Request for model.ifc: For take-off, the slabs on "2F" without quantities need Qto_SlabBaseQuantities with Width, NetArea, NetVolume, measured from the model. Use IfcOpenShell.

First a look at what the model holds.

```python
import ifcopenshell
import ifcopenshell.util.element
import ifcopenshell.util.unit

model = ifcopenshell.open("model.ifc")
print(model.schema)
for unit_type in ("LENGTHUNIT", "AREAUNIT", "VOLUMEUNIT"):
    print(unit_type, ifcopenshell.util.unit.calculate_unit_scale(model, unit_type))
storey = next(s for s in model.by_type("IfcBuildingStorey") if s.Name == "2F")
slabs = [e for e in ifcopenshell.util.element.get_decomposition(storey) if e.is_a("IfcSlab")]
for e in sorted(slabs, key=lambda e: e.id()):
    print(e.id(), e.is_a(), e.Name, list(ifcopenshell.util.element.get_psets(e, qtos_only=True)), sep=" | ")
```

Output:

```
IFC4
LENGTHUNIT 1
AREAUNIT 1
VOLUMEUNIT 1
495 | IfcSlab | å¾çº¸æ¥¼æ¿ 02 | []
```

```python
import ifcopenshell
import ifcopenshell.api.pset
import ifcopenshell.geom
import ifcopenshell.util.element
import ifcopenshell.util.shape
import ifcopenshell.util.unit

model = ifcopenshell.open("model.ifc")
unit_scale = ifcopenshell.util.unit.calculate_unit_scale(model)
area_scale = ifcopenshell.util.unit.calculate_unit_scale(model, "AREAUNIT")
volume_scale = ifcopenshell.util.unit.calculate_unit_scale(model, "VOLUMEUNIT")
settings = ifcopenshell.geom.settings()

storey = next(s for s in model.by_type("IfcBuildingStorey") if s.Name == "2F")
slabs = [e for e in ifcopenshell.util.element.get_decomposition(storey) if e.is_a("IfcSlab")]

for e in sorted(slabs, key=lambda e: e.id()):
    if ifcopenshell.util.element.get_psets(e, qtos_only=True, should_inherit=False):
        continue
    # Geometry comes back in metres, in the element's own axes.
    shape = ifcopenshell.geom.create_shape(settings, e)
    values = {
        "Width": ifcopenshell.util.shape.get_z(shape.geometry) / unit_scale,
        "NetArea": ifcopenshell.util.shape.get_footprint_area(shape.geometry) / area_scale,
        "NetVolume": ifcopenshell.util.shape.get_volume(shape.geometry) / volume_scale,
    }
    qto = ifcopenshell.api.pset.add_qto(model, product=e, name="Qto_SlabBaseQuantities")
    ifcopenshell.api.pset.edit_qto(model, qto=qto, properties=values)
    print(e.id(), {k: round(v, 3) for k, v in values.items()})

model.write("model_edited.ifc")
```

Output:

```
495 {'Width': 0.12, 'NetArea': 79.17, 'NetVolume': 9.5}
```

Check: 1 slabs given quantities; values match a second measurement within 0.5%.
